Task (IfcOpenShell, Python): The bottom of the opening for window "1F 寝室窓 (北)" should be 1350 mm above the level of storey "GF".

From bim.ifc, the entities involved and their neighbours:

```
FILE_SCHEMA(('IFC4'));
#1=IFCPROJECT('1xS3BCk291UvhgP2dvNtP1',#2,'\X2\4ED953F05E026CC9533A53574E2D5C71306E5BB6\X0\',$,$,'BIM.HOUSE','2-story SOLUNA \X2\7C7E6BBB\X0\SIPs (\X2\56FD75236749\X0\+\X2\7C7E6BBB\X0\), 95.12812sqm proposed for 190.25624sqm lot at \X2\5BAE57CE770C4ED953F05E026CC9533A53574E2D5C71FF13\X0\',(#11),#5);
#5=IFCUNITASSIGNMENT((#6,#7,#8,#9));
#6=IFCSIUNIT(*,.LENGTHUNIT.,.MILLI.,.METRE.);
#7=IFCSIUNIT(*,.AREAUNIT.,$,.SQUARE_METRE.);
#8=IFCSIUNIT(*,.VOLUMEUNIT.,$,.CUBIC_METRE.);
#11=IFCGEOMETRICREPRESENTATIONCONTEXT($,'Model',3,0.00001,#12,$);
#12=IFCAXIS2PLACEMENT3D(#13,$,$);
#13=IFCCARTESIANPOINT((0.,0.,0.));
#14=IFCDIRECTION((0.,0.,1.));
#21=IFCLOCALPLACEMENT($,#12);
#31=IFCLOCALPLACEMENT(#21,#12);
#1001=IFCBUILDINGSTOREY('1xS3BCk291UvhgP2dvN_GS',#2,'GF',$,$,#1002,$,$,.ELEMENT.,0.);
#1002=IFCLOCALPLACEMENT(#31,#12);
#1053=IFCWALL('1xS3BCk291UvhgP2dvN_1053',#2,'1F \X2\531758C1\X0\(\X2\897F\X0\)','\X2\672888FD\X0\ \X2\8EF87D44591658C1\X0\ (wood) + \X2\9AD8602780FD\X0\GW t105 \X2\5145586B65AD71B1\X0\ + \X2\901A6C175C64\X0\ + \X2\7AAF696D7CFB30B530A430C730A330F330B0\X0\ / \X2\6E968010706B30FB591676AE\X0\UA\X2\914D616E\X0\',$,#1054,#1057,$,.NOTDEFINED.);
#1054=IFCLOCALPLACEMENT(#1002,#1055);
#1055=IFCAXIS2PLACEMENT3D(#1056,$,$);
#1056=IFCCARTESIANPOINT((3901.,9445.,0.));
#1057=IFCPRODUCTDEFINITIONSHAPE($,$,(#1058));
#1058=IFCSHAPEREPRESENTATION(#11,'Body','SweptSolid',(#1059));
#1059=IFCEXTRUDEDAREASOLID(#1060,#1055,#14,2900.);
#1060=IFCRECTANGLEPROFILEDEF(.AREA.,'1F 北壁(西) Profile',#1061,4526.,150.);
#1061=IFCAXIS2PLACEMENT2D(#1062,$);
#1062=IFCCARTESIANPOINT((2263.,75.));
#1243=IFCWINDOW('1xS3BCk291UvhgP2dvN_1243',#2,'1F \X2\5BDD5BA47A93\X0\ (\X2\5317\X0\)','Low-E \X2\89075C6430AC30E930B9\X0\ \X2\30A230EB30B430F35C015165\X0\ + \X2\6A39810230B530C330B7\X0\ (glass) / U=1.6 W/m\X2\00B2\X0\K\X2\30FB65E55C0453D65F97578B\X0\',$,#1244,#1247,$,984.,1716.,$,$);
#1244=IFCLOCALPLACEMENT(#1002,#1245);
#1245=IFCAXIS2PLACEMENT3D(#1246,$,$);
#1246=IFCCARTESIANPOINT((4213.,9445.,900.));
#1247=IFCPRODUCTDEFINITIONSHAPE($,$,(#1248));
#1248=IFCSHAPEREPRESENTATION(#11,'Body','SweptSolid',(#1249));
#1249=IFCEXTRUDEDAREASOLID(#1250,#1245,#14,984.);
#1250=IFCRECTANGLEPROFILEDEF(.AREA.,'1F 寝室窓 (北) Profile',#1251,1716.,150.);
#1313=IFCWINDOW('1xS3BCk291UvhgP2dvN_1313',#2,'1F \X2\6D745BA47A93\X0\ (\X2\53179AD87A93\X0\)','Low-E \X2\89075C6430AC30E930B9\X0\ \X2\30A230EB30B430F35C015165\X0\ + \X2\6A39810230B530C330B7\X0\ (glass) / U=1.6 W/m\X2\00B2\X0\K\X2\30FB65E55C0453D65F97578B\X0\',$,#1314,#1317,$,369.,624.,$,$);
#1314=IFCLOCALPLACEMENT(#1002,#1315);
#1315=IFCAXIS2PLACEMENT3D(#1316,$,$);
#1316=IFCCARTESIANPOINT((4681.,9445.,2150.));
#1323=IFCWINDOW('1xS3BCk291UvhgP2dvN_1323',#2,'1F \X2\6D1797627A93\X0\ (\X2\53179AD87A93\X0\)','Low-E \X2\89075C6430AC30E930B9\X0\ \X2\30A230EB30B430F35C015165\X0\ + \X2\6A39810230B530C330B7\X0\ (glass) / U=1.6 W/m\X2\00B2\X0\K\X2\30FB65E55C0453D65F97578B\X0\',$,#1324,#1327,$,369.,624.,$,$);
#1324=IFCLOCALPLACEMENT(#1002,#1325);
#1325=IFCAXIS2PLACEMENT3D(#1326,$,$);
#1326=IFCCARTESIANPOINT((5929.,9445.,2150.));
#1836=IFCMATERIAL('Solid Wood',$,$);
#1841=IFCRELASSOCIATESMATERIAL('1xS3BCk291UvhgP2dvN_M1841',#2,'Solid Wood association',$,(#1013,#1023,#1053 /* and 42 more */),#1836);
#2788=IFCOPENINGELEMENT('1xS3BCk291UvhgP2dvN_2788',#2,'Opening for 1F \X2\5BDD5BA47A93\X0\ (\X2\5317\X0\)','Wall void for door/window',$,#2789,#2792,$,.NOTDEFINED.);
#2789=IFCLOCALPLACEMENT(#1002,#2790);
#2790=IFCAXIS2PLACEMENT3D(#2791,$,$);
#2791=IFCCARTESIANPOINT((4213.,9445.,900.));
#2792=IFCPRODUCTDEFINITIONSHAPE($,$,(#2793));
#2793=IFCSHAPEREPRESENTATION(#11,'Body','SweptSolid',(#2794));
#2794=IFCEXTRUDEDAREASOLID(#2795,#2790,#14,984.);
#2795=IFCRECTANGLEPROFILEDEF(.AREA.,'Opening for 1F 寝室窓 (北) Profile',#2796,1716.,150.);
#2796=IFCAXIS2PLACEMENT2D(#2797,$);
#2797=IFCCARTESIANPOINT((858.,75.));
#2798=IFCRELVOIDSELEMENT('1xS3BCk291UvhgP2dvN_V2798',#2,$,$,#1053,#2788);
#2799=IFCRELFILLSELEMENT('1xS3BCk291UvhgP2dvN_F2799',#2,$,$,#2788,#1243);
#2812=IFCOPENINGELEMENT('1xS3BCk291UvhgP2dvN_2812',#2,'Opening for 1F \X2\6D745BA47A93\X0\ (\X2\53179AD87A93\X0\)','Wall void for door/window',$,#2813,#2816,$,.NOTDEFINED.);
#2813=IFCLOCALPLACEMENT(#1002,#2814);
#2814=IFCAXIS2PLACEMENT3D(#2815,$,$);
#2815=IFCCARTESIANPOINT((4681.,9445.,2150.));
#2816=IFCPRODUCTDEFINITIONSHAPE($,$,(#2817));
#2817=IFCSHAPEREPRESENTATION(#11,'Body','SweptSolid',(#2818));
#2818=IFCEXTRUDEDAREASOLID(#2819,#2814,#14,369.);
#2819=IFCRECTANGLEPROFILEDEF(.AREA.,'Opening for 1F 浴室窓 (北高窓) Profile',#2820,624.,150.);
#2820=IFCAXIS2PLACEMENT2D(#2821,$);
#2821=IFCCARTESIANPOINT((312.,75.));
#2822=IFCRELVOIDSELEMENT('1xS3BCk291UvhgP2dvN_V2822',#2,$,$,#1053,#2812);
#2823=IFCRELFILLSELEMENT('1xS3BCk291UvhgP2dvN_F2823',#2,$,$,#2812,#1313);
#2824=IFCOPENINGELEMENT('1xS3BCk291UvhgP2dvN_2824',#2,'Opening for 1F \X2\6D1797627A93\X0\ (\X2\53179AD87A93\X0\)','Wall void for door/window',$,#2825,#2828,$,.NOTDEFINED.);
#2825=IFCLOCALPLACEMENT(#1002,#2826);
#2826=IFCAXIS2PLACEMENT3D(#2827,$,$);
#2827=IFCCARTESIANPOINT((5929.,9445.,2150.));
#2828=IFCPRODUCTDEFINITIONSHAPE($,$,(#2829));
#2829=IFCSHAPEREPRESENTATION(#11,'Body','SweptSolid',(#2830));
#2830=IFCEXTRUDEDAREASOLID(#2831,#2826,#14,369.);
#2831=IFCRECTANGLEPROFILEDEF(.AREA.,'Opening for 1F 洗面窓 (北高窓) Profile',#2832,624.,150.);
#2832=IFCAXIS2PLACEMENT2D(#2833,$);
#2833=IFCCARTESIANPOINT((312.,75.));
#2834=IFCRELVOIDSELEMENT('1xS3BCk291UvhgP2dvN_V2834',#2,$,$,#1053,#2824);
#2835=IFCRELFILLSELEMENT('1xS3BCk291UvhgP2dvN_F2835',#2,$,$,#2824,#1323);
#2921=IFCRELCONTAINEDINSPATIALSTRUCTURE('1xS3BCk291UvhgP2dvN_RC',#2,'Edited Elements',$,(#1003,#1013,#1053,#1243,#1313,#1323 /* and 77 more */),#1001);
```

```python
import numpy as np
import ifcopenshell
import ifcopenshell.api.geometry
import ifcopenshell.geom
import ifcopenshell.util.element
import ifcopenshell.util.placement
import ifcopenshell.util.shape
import ifcopenshell.util.unit

model = ifcopenshell.open("bim.ifc")
unit_scale = ifcopenshell.util.unit.calculate_unit_scale(model)

window = model.by_guid("1xS3BCk291UvhgP2dvN_1243")
opening = window.FillsVoids[0].RelatingOpeningElement
storey = ifcopenshell.util.element.get_container(window, ifc_class="IfcBuildingStorey")
level = ifcopenshell.util.placement.get_local_placement(storey.ObjectPlacement)[2, 3]

# The opening's origin need not be at the sill, so measure its lowest point.
shape = ifcopenshell.geom.create_shape(ifcopenshell.geom.settings(), opening)
bottom = ifcopenshell.util.shape.get_shape_bottom_elevation(shape, shape.geometry) / unit_scale
dz = level + 1.35 / unit_scale - bottom

shift = np.array([0.0, 0.0, dz])
# The window is not placed relative to its opening, so move both.
for product in (opening, window):
    matrix = ifcopenshell.util.placement.get_local_placement(product.ObjectPlacement)
    matrix[:3, 3] += shift
    ifcopenshell.api.geometry.edit_object_placement(model, product=product, matrix=matrix, is_si=False)

print(f"moved by {dz * unit_scale:+.3f} m")

model.write("bim_edited.ifc")
```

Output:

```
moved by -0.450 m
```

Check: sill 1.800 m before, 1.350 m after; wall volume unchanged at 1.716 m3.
